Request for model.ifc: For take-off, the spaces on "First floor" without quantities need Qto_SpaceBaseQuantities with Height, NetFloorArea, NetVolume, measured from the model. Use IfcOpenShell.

First a look at what the model holds.

```python
import ifcopenshell
import ifcopenshell.util.element
import ifcopenshell.util.unit

model = ifcopenshell.open("model.ifc")
print(model.schema)
for unit_type in ("LENGTHUNIT", "AREAUNIT", "VOLUMEUNIT"):
    print(unit_type, ifcopenshell.util.unit.calculate_unit_scale(model, unit_type))
storey = next(s for s in model.by_type("IfcBuildingStorey") if s.Name == "First floor")
spaces = [e for e in ifcopenshell.util.element.get_decomposition(storey) if e.is_a("IfcSpace")]
for e in sorted(spaces, key=lambda e: e.id()):
    print(e.id(), e.is_a(), e.Name, list(ifcopenshell.util.element.get_psets(e, qtos_only=True)), sep=" | ")
```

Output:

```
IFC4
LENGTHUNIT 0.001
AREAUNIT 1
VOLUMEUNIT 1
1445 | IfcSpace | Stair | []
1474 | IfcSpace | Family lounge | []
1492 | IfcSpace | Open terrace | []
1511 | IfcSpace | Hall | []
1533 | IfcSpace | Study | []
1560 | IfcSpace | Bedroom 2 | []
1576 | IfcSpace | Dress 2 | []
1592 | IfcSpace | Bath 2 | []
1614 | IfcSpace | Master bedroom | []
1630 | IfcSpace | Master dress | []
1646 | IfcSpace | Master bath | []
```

```python
import ifcopenshell
import ifcopenshell.api.pset
import ifcopenshell.geom
import ifcopenshell.util.element
import ifcopenshell.util.shape
import ifcopenshell.util.unit

model = ifcopenshell.open("model.ifc")
unit_scale = ifcopenshell.util.unit.calculate_unit_scale(model)
area_scale = ifcopenshell.util.unit.calculate_unit_scale(model, "AREAUNIT")
volume_scale = ifcopenshell.util.unit.calculate_unit_scale(model, "VOLUMEUNIT")
settings = ifcopenshell.geom.settings()

storey = next(s for s in model.by_type("IfcBuildingStorey") if s.Name == "First floor")
spaces = [e for e in ifcopenshell.util.element.get_decomposition(storey) if e.is_a("IfcSpace")]

for e in sorted(spaces, key=lambda e: e.id()):
    if ifcopenshell.util.element.get_psets(e, qtos_only=True, should_inherit=False):
        continue
    # Geometry comes back in metres, in the element's own axes.
    shape = ifcopenshell.geom.create_shape(settings, e)
    values = {
        "Height": ifcopenshell.util.shape.get_z(shape.geometry) / unit_scale,
        "NetFloorArea": ifcopenshell.util.shape.get_footprint_area(shape.geometry) / area_scale,
        "NetVolume": ifcopenshell.util.shape.get_volume(shape.geometry) / volume_scale,
    }
    qto = ifcopenshell.api.pset.add_qto(model, product=e, name="Qto_SpaceBaseQuantities")
    ifcopenshell.api.pset.edit_qto(model, qto=qto, properties=values)
    print(e.id(), {k: round(v, 3) for k, v in values.items()})

model.write("model-out.ifc")
```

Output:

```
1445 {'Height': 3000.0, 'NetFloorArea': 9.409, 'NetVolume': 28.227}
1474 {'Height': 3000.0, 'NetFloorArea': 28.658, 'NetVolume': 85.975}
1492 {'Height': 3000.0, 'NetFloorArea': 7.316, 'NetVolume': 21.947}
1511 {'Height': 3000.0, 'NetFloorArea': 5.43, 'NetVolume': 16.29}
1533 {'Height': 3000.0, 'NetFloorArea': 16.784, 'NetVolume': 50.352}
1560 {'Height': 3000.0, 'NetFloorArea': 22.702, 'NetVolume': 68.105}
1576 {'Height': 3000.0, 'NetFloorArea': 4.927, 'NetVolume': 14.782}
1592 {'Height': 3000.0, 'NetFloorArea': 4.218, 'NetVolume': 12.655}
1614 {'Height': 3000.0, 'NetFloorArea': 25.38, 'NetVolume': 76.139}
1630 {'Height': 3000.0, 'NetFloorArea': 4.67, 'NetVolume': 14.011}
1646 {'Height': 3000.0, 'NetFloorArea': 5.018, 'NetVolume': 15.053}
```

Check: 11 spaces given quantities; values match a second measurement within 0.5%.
